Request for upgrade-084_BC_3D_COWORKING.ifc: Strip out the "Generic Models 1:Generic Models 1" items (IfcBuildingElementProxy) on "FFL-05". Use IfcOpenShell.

First a look at what the model holds.

```python
import ifcopenshell
import ifcopenshell.util.element

model = ifcopenshell.open("upgrade-084_BC_3D_COWORKING.ifc")
print(model.schema)
storey = next(s for s in model.by_type("IfcBuildingStorey") if s.Name == "FFL-05")
proxies = [e for e in ifcopenshell.util.element.get_decomposition(storey) if e.is_a("IfcBuildingElementProxy")]
seen = {}
for e in proxies:
    element_type = ifcopenshell.util.element.get_type(e)
    name = element_type.Name if element_type not in (None, e) else None
    seen[name] = seen.get(name, 0) + 1
for name, count in sorted(seen.items(), key=str):
    print(count, "x", name)
```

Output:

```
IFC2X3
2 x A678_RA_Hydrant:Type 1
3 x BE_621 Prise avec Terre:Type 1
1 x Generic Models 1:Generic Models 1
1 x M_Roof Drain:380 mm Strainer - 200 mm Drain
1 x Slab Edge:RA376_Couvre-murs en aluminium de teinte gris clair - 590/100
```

```python
import ifcopenshell
import ifcopenshell.api.root
import ifcopenshell.util.element

model = ifcopenshell.open("upgrade-084_BC_3D_COWORKING.ifc")

storey = next(s for s in model.by_type("IfcBuildingStorey") if s.Name == "FFL-05")
proxies = [e for e in ifcopenshell.util.element.get_decomposition(storey) if e.is_a("IfcBuildingElementProxy")]
targets = [e for e in proxies if (t := ifcopenshell.util.element.get_type(e)) not in (None, e) and t.Name == "Generic Models 1:Generic Models 1"]

for e in targets:
    ifcopenshell.api.root.remove_product(model, product=e)
print(len(targets), "removed")

model.write("upgrade-084_BC_3D_COWORKING_updated.ifc")
```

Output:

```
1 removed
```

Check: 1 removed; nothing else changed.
